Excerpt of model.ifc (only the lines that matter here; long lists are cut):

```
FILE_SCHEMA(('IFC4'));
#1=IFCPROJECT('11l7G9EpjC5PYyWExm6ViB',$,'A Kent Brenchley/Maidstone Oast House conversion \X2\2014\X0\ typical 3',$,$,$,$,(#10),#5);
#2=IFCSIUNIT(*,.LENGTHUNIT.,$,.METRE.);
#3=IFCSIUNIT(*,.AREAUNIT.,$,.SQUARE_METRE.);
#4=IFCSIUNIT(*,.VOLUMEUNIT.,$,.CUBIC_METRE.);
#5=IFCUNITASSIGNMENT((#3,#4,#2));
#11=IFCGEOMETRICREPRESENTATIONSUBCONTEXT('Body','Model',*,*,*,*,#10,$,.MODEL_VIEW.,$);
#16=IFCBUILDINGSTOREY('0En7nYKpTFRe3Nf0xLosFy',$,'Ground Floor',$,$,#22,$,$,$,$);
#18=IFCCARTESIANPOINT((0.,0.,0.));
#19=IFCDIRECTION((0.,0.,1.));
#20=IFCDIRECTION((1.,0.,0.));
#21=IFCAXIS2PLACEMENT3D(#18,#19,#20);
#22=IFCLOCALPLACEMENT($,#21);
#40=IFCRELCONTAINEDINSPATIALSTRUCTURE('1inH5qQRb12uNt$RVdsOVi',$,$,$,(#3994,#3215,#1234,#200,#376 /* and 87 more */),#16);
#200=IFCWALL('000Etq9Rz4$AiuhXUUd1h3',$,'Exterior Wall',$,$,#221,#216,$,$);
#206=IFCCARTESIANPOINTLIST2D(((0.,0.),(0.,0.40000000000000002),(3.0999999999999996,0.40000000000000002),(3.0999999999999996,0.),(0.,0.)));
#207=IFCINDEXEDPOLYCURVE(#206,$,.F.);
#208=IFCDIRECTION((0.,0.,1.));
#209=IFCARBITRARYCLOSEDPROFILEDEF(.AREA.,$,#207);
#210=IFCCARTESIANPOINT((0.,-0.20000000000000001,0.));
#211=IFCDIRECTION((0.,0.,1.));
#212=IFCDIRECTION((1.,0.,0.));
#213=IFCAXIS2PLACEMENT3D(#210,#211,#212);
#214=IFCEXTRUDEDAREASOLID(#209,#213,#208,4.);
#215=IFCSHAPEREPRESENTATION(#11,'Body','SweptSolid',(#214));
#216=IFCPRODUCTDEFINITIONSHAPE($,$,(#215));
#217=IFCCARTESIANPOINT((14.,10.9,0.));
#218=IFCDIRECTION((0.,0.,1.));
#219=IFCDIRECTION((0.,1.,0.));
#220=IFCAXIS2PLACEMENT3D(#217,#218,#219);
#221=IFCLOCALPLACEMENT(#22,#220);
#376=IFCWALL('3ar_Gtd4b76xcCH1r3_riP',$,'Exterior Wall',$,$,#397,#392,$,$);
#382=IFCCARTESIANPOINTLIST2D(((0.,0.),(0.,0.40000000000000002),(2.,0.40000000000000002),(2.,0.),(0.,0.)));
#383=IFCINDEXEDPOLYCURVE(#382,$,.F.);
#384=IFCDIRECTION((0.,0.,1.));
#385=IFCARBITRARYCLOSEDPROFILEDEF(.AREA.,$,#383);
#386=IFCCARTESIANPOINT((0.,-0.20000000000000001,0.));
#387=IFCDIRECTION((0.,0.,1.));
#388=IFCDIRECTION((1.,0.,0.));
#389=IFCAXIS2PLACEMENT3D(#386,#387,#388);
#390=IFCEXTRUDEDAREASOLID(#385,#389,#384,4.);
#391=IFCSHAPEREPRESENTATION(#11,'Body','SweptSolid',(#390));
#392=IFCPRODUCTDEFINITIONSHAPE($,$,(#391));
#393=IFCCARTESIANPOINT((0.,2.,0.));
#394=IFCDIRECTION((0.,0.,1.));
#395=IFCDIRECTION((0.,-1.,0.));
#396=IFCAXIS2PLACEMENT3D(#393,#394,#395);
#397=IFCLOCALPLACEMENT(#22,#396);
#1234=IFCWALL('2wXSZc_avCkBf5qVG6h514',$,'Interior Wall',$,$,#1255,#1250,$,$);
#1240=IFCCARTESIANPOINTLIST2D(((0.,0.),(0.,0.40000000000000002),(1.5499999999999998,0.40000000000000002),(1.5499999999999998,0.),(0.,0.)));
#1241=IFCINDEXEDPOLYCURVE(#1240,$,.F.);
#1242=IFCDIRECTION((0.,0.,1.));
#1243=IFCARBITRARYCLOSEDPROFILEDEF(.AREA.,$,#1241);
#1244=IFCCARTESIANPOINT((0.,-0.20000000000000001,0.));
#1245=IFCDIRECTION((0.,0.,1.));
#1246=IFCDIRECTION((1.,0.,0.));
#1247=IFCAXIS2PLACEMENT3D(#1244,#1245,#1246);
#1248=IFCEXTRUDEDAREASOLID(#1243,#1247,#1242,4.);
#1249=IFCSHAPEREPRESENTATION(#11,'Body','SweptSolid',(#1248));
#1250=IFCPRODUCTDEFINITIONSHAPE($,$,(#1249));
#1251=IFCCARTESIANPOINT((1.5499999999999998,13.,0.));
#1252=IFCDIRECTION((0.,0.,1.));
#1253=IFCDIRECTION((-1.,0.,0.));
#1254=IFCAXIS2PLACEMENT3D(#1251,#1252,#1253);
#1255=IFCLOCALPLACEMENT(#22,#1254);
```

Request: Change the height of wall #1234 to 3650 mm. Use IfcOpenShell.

```python
import ifcopenshell
import ifcopenshell.geom
import ifcopenshell.util.representation
import ifcopenshell.util.shape

model = ifcopenshell.open("model.ifc")
settings = ifcopenshell.geom.settings()


def volume(element):
    """Net volume in cubic metres, openings subtracted."""
    shape = ifcopenshell.geom.create_shape(settings, element)
    return ifcopenshell.util.shape.get_volume(shape.geometry)


wall = model.by_guid("2wXSZc_avCkBf5qVG6h514")
before = volume(wall)

body = ifcopenshell.util.representation.get_representation(wall, "Model", "Body")
solid = body.Items[0]
old_height = solid.Depth
solid.Depth = 3.65
after = volume(wall)

print(f"height {old_height:g} -> {solid.Depth:g}, volume {before:.3f} -> {after:.3f} m3")

model.write("model_edited.ifc")
```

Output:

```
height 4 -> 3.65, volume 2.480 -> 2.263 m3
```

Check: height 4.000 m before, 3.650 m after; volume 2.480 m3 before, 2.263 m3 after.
